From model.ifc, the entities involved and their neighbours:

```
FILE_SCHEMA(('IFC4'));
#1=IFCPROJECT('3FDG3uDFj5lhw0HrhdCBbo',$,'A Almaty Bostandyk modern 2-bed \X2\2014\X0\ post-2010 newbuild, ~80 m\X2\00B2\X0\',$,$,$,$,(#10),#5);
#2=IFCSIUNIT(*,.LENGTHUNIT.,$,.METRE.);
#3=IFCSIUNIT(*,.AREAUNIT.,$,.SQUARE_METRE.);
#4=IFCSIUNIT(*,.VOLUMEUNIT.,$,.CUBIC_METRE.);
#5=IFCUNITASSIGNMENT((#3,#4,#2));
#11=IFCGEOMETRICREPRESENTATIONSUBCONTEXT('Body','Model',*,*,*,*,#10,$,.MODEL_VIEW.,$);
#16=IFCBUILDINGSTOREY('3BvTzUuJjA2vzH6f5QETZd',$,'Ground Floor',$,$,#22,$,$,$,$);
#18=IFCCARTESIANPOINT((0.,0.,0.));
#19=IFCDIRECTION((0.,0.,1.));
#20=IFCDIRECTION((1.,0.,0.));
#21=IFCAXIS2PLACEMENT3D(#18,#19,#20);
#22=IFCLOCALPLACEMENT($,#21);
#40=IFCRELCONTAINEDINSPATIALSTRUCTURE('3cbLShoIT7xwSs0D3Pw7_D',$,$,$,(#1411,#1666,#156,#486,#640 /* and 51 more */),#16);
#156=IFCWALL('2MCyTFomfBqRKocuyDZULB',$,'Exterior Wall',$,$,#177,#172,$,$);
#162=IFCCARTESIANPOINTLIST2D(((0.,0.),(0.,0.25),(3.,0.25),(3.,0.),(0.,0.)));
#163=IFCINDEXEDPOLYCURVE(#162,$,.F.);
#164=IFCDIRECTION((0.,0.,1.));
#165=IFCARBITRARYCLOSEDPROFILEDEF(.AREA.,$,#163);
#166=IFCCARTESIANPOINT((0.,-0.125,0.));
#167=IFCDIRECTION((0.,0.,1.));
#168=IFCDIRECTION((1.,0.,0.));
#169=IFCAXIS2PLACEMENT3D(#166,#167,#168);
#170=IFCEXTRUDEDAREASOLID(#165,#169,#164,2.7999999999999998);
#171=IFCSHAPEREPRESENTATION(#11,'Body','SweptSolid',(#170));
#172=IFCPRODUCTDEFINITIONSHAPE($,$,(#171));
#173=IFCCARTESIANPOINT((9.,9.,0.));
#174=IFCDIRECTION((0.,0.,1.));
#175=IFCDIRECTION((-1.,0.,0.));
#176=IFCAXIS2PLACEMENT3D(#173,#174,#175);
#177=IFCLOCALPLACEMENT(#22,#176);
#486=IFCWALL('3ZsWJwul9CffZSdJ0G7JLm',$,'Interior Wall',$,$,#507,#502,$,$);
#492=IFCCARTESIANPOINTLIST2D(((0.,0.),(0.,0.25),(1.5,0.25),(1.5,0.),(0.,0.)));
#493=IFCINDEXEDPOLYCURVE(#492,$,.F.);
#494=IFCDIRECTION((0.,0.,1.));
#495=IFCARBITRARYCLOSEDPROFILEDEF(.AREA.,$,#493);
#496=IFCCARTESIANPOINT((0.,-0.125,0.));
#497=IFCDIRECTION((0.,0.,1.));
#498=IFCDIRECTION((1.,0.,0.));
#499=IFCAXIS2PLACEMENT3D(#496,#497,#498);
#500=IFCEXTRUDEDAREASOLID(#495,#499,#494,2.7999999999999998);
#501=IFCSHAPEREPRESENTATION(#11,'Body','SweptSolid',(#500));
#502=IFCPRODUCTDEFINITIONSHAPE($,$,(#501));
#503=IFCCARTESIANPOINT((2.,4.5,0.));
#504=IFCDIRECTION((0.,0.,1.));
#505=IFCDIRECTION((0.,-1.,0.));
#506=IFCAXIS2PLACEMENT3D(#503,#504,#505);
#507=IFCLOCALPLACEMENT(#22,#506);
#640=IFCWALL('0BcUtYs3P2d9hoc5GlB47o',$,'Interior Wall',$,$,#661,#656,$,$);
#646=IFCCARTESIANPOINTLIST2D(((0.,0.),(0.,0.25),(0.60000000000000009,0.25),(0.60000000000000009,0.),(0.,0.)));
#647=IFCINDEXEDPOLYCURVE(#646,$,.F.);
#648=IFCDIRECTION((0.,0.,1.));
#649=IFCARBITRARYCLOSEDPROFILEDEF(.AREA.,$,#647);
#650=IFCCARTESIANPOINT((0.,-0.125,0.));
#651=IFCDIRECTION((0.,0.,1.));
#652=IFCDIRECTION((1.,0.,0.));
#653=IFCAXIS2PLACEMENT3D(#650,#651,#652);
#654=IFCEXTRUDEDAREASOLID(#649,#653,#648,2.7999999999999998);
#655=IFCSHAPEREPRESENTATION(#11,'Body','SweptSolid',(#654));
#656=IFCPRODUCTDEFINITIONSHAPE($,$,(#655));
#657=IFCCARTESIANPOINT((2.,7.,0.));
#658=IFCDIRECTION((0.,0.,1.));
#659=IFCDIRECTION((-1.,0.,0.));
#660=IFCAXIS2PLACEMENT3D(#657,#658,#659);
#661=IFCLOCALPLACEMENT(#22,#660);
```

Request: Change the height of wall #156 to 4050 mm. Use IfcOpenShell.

```python
import ifcopenshell
import ifcopenshell.geom
import ifcopenshell.util.representation
import ifcopenshell.util.shape

model = ifcopenshell.open("model.ifc")
settings = ifcopenshell.geom.settings()


def volume(element):
    """Net volume in cubic metres, openings subtracted."""
    shape = ifcopenshell.geom.create_shape(settings, element)
    return ifcopenshell.util.shape.get_volume(shape.geometry)


wall = model.by_guid("2MCyTFomfBqRKocuyDZULB")
before = volume(wall)

body = ifcopenshell.util.representation.get_representation(wall, "Model", "Body")
solid = body.Items[0]
old_height = solid.Depth
solid.Depth = 4.05
after = volume(wall)

print(f"height {old_height:g} -> {solid.Depth:g}, volume {before:.3f} -> {after:.3f} m3")

model.write("model_v2.ifc")
```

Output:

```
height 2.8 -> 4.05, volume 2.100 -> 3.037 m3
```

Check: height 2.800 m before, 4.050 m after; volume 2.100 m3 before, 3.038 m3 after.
